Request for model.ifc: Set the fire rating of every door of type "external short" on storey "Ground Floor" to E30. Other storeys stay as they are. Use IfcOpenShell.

First a look at what the model holds.

```python
import ifcopenshell
import ifcopenshell.util.element

model = ifcopenshell.open("model.ifc")
print(model.schema)
storey = next(s for s in model.by_type("IfcBuildingStorey") if s.Name == "Ground Floor")
doors = [e for e in ifcopenshell.util.element.get_decomposition(storey) if e.is_a("IfcDoor")]
seen = {}
for e in doors:
    element_type = ifcopenshell.util.element.get_type(e)
    key = (element_type.Name if element_type != e and element_type else None, ifcopenshell.util.element.get_pset(e, "Pset_DoorCommon", "FireRating"))
    seen[key] = seen.get(key, 0) + 1
for (name, value), count in sorted(seen.items(), key=str):
    print(count, "x", name, "|", value)
```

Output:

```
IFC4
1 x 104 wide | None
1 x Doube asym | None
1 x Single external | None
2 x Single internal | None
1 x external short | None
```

```python
import ifcopenshell
import ifcopenshell.api.pset
import ifcopenshell.util.element

model = ifcopenshell.open("model.ifc")

storey = next(s for s in model.by_type("IfcBuildingStorey") if s.Name == "Ground Floor")
doors = [e for e in ifcopenshell.util.element.get_decomposition(storey) if e.is_a("IfcDoor")]

count = 0
for e in doors:
    element_type = ifcopenshell.util.element.get_type(e)
    if element_type in (None, e) or element_type.Name != "external short":
        continue
    # add_pset returns the element's existing set when there is one.
    pset = ifcopenshell.api.pset.add_pset(model, product=e, name="Pset_DoorCommon")
    ifcopenshell.api.pset.edit_pset(model, pset=pset, properties={"FireRating": "E30"})
    count += 1

print(count, "doors updated")

model.write("model_edited.ifc")
```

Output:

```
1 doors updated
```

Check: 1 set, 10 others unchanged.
